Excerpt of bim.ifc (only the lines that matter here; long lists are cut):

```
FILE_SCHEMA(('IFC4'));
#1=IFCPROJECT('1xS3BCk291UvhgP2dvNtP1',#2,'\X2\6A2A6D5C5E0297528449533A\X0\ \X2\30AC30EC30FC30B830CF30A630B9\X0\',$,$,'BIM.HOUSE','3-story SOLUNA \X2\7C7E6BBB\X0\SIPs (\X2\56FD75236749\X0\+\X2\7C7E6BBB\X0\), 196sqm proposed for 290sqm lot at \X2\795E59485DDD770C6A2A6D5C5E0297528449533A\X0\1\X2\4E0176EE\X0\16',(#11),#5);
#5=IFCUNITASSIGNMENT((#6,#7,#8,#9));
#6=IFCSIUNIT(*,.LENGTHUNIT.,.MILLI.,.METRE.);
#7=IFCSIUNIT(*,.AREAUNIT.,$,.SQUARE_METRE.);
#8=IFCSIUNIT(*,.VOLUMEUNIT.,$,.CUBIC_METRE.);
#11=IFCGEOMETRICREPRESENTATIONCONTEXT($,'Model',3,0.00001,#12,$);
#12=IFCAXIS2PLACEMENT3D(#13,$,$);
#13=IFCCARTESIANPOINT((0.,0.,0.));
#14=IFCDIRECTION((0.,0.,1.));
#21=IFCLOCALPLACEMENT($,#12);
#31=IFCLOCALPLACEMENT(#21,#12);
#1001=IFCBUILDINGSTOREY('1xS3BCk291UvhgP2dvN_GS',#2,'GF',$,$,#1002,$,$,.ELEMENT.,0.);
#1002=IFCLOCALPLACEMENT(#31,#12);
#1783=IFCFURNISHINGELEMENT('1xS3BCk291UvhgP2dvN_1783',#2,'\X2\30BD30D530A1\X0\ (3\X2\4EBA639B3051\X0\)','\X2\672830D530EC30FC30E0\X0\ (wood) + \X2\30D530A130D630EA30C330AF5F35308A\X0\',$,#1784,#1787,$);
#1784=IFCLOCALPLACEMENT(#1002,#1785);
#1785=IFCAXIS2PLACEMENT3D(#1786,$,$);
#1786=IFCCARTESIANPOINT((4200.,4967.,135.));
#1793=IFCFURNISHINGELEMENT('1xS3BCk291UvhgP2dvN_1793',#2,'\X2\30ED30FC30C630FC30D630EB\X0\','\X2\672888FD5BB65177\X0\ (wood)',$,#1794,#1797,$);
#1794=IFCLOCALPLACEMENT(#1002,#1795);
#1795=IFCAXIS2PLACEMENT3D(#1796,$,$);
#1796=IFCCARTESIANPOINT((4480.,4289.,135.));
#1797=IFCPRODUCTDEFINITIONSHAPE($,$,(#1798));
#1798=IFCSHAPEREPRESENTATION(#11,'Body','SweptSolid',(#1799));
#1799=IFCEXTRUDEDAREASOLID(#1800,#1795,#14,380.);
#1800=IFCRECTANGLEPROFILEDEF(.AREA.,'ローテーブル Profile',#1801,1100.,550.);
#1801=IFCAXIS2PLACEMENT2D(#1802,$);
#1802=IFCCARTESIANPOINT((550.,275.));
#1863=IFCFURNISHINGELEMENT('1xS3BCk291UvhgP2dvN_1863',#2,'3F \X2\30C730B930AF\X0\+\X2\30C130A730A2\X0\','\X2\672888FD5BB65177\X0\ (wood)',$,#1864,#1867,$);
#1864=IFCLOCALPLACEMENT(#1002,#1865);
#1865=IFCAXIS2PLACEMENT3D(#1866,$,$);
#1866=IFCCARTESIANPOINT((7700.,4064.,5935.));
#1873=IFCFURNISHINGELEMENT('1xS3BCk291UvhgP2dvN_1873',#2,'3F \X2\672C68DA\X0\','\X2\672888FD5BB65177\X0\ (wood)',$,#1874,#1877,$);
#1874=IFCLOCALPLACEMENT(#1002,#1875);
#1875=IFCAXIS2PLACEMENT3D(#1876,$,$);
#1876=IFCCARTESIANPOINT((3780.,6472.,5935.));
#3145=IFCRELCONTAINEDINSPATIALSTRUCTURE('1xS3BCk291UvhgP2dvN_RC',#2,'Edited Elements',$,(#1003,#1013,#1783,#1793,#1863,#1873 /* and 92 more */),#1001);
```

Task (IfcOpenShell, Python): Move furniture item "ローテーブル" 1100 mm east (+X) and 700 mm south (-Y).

```python
import ifcopenshell
import ifcopenshell.api.geometry
import ifcopenshell.util.placement
import ifcopenshell.util.unit

model = ifcopenshell.open("bim.ifc")
unit_scale = ifcopenshell.util.unit.calculate_unit_scale(model)

item = model.by_guid("1xS3BCk291UvhgP2dvN_1793")
matrix = ifcopenshell.util.placement.get_local_placement(item.ObjectPlacement)
matrix[0, 3] += 1.1 / unit_scale
matrix[1, 3] -= 0.7 / unit_scale
ifcopenshell.api.geometry.edit_object_placement(model, product=item, matrix=matrix, is_si=False)

print(ifcopenshell.util.placement.get_local_placement(item.ObjectPlacement).round(3) + 0.0)

model.write("bim_v2.ifc")
```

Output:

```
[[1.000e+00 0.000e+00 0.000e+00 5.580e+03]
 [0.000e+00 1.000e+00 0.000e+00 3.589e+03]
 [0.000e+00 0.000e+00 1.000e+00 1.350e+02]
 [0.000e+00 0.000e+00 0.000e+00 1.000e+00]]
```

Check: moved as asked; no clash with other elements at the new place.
